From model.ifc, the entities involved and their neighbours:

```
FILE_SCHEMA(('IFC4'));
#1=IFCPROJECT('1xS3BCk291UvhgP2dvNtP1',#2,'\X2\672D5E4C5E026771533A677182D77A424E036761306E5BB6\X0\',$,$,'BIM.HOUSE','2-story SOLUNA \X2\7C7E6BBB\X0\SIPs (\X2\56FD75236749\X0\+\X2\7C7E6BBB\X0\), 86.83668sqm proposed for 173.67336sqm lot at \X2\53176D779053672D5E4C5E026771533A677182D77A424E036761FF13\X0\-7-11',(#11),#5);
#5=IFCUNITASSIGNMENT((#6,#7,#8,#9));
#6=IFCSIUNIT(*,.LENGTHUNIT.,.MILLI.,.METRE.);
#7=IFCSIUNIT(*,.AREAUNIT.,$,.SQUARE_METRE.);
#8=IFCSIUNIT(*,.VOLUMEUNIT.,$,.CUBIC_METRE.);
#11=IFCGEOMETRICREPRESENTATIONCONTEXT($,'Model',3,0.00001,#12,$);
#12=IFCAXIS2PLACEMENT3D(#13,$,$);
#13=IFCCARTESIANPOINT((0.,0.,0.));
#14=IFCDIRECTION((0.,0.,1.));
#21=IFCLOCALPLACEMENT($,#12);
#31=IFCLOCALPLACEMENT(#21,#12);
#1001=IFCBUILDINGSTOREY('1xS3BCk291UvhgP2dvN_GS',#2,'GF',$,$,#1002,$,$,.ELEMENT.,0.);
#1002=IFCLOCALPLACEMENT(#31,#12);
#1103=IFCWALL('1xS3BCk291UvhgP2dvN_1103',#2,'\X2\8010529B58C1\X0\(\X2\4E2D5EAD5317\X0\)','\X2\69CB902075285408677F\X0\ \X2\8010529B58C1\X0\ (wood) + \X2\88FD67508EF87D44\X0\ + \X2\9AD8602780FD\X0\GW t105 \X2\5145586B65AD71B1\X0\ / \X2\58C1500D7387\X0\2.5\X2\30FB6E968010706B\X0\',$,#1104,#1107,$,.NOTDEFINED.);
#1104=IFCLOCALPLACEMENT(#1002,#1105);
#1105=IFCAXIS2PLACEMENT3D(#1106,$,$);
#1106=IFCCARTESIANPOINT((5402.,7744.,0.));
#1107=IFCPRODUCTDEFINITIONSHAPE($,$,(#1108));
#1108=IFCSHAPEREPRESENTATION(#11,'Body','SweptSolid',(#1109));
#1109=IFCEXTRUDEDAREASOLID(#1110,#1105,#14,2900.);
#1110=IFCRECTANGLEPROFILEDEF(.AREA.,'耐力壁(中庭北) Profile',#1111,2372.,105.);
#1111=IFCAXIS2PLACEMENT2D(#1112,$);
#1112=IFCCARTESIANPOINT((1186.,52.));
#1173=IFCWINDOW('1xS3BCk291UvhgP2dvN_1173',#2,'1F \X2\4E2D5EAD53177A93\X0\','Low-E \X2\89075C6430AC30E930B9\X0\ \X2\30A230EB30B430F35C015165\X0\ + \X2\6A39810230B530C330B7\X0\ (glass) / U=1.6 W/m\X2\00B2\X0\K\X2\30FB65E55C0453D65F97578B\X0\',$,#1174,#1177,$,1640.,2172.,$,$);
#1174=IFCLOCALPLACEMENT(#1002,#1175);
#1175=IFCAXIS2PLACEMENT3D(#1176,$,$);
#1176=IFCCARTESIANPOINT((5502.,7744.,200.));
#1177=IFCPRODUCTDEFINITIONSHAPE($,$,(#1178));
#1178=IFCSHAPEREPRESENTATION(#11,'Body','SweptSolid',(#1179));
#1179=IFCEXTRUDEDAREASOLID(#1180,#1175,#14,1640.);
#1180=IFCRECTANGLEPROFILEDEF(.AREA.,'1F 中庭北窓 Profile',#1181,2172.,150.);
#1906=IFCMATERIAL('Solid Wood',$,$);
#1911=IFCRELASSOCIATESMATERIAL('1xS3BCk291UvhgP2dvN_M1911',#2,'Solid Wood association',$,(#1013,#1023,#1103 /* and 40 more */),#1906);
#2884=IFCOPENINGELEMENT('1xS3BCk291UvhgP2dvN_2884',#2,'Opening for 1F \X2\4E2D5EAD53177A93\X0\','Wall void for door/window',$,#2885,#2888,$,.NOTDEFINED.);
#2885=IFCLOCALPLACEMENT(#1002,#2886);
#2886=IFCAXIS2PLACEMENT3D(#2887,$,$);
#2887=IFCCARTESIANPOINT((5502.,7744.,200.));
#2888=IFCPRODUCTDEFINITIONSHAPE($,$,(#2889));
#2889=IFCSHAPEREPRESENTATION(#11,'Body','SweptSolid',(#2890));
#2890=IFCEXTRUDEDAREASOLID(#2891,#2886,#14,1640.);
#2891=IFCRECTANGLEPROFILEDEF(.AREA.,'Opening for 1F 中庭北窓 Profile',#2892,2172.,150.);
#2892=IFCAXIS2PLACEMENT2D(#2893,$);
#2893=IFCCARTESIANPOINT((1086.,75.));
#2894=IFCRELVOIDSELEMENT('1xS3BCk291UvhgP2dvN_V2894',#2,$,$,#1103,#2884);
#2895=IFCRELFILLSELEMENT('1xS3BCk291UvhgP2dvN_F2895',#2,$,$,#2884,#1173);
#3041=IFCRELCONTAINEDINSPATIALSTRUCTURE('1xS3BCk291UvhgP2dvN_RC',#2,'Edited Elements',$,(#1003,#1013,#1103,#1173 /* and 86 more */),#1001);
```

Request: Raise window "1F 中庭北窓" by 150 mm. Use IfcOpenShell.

```python
import numpy as np
import ifcopenshell
import ifcopenshell.api.geometry
import ifcopenshell.util.placement
import ifcopenshell.util.unit

model = ifcopenshell.open("model.ifc")
unit_scale = ifcopenshell.util.unit.calculate_unit_scale(model)

window = model.by_guid("1xS3BCk291UvhgP2dvN_1173")
opening = window.FillsVoids[0].RelatingOpeningElement
dz = 0.15 / unit_scale

shift = np.array([0.0, 0.0, dz])
# The window is not placed relative to its opening, so move both.
for product in (opening, window):
    matrix = ifcopenshell.util.placement.get_local_placement(product.ObjectPlacement)
    matrix[:3, 3] += shift
    ifcopenshell.api.geometry.edit_object_placement(model, product=product, matrix=matrix, is_si=False)

print(f"moved by {dz * unit_scale:+.3f} m")

model.write("model_edited.ifc")
```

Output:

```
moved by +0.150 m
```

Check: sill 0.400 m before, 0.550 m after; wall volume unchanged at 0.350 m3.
